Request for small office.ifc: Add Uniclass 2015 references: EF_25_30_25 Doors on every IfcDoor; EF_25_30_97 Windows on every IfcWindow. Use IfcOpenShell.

First a look at what the model holds.

```python
import ifcopenshell

model = ifcopenshell.open("small office.ifc")
print(model.schema)
print("classifications:", [c.Name for c in model.by_type("IfcClassification")])
for ifc_class in ("IfcDoor", "IfcRoof", "IfcStair", "IfcWall", "IfcWindow"):
    print(ifc_class, len(model.by_type(ifc_class)))
```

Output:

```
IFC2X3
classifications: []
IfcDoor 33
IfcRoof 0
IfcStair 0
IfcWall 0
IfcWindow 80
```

```python
import ifcopenshell
import ifcopenshell.api.classification

model = ifcopenshell.open("small office.ifc")

# IFC2X3 requires Source and Edition and has no link from the project to the system.
system = model.create_entity("IfcClassification", Source="NBS", Edition="2015", Name="Uniclass 2015")

codes = {
    "IfcDoor": ("EF_25_30_25", "Doors"),
    "IfcWindow": ("EF_25_30_97", "Windows"),
}
for ifc_class, (code, name) in codes.items():
    products = model.by_type(ifc_class)
    ifcopenshell.api.classification.add_reference(
        model, products=products, classification=system, identification=code, name=name
    )
    print(code, len(products))

model.write("small office_rev.ifc")
```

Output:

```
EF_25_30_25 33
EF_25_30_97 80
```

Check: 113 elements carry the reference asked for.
